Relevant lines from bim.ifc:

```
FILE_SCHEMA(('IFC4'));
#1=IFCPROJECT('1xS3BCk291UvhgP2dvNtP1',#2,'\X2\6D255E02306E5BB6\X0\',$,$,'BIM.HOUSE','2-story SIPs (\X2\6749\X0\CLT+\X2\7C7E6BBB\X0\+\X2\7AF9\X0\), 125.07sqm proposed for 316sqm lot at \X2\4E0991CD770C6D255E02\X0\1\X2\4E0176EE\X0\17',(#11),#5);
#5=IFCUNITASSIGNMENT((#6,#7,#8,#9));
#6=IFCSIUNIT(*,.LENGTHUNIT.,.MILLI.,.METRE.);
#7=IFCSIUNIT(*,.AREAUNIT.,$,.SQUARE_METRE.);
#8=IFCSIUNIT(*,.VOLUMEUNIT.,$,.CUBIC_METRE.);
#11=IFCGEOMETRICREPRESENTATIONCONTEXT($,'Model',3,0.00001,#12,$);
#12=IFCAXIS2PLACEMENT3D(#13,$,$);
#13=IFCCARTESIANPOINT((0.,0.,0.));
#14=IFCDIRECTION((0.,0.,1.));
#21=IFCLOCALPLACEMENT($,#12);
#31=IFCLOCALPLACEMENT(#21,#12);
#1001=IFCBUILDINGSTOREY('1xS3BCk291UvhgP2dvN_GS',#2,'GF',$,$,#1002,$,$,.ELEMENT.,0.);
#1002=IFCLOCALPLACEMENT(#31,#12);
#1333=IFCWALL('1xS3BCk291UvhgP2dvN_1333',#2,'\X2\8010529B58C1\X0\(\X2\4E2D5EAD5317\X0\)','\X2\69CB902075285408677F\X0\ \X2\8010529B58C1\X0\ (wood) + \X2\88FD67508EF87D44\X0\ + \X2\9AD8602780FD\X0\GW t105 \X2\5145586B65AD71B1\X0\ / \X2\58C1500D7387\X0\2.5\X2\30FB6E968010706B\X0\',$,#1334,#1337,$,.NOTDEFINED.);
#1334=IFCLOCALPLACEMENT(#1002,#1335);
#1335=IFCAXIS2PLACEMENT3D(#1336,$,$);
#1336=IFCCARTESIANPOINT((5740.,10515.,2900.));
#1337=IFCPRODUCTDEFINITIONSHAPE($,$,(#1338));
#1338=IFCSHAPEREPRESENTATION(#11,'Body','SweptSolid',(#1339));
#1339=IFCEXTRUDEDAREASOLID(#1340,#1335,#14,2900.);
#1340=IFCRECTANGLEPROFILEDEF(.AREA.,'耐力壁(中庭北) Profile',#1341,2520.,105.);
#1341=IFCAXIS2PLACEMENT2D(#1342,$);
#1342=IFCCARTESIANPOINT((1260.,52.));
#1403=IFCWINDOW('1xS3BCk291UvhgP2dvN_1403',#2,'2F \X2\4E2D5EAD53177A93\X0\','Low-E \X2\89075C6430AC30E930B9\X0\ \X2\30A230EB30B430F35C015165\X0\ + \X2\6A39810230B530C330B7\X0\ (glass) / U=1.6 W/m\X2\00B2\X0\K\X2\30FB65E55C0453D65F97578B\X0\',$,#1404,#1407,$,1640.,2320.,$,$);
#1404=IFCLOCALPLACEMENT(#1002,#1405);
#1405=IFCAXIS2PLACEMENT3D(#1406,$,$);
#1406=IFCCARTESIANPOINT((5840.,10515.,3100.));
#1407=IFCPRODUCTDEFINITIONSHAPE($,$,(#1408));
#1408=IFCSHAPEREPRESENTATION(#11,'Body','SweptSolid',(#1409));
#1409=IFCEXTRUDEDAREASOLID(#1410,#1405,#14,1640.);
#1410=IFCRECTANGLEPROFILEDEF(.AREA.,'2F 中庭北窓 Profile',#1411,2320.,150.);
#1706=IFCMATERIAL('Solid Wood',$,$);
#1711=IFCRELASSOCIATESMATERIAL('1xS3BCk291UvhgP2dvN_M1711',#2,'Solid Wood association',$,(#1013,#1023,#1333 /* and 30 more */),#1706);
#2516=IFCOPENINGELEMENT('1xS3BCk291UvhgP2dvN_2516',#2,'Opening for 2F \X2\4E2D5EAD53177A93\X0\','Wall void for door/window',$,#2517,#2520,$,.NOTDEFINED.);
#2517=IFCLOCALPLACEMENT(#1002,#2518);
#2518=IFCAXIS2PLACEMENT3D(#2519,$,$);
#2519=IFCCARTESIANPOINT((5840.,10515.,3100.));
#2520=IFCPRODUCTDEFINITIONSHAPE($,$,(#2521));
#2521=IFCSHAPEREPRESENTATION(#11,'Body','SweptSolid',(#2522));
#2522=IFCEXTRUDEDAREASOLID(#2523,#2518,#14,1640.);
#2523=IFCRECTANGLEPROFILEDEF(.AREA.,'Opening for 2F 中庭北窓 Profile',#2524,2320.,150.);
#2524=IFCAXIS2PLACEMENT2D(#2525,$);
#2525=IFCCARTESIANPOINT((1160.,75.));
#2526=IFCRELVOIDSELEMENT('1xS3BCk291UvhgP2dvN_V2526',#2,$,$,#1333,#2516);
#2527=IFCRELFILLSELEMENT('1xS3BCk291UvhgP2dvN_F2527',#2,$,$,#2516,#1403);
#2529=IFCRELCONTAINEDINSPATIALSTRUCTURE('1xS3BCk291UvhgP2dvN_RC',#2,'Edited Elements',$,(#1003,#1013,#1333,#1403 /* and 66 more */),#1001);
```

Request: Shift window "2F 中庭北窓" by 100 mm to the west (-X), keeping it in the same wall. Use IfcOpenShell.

```python
import ifcopenshell
import ifcopenshell.api.geometry
import ifcopenshell.util.placement
import ifcopenshell.util.unit

model = ifcopenshell.open("bim.ifc")
unit_scale = ifcopenshell.util.unit.calculate_unit_scale(model)

window = model.by_guid("1xS3BCk291UvhgP2dvN_1403")
opening = window.FillsVoids[0].RelatingOpeningElement
wall = opening.VoidsElements[0].RelatingBuildingElement

wall_matrix = ifcopenshell.util.placement.get_local_placement(wall.ObjectPlacement)
shift = wall_matrix[:3, 0] * -0.1 / unit_scale
before = ifcopenshell.util.placement.get_local_placement(window.ObjectPlacement)[:3, 3].copy()

# The window is not placed relative to its opening, so move both.
for product in (opening, window):
    matrix = ifcopenshell.util.placement.get_local_placement(product.ObjectPlacement)
    matrix[:3, 3] += shift
    ifcopenshell.api.geometry.edit_object_placement(model, product=product, matrix=matrix, is_si=False)

after = ifcopenshell.util.placement.get_local_placement(window.ObjectPlacement)[:3, 3]
print("window moved by", (after - before).round(3) + 0.0)

model.write("bim_edited.ifc")
```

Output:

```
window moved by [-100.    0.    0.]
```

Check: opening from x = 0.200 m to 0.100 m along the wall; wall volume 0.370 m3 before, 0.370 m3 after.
